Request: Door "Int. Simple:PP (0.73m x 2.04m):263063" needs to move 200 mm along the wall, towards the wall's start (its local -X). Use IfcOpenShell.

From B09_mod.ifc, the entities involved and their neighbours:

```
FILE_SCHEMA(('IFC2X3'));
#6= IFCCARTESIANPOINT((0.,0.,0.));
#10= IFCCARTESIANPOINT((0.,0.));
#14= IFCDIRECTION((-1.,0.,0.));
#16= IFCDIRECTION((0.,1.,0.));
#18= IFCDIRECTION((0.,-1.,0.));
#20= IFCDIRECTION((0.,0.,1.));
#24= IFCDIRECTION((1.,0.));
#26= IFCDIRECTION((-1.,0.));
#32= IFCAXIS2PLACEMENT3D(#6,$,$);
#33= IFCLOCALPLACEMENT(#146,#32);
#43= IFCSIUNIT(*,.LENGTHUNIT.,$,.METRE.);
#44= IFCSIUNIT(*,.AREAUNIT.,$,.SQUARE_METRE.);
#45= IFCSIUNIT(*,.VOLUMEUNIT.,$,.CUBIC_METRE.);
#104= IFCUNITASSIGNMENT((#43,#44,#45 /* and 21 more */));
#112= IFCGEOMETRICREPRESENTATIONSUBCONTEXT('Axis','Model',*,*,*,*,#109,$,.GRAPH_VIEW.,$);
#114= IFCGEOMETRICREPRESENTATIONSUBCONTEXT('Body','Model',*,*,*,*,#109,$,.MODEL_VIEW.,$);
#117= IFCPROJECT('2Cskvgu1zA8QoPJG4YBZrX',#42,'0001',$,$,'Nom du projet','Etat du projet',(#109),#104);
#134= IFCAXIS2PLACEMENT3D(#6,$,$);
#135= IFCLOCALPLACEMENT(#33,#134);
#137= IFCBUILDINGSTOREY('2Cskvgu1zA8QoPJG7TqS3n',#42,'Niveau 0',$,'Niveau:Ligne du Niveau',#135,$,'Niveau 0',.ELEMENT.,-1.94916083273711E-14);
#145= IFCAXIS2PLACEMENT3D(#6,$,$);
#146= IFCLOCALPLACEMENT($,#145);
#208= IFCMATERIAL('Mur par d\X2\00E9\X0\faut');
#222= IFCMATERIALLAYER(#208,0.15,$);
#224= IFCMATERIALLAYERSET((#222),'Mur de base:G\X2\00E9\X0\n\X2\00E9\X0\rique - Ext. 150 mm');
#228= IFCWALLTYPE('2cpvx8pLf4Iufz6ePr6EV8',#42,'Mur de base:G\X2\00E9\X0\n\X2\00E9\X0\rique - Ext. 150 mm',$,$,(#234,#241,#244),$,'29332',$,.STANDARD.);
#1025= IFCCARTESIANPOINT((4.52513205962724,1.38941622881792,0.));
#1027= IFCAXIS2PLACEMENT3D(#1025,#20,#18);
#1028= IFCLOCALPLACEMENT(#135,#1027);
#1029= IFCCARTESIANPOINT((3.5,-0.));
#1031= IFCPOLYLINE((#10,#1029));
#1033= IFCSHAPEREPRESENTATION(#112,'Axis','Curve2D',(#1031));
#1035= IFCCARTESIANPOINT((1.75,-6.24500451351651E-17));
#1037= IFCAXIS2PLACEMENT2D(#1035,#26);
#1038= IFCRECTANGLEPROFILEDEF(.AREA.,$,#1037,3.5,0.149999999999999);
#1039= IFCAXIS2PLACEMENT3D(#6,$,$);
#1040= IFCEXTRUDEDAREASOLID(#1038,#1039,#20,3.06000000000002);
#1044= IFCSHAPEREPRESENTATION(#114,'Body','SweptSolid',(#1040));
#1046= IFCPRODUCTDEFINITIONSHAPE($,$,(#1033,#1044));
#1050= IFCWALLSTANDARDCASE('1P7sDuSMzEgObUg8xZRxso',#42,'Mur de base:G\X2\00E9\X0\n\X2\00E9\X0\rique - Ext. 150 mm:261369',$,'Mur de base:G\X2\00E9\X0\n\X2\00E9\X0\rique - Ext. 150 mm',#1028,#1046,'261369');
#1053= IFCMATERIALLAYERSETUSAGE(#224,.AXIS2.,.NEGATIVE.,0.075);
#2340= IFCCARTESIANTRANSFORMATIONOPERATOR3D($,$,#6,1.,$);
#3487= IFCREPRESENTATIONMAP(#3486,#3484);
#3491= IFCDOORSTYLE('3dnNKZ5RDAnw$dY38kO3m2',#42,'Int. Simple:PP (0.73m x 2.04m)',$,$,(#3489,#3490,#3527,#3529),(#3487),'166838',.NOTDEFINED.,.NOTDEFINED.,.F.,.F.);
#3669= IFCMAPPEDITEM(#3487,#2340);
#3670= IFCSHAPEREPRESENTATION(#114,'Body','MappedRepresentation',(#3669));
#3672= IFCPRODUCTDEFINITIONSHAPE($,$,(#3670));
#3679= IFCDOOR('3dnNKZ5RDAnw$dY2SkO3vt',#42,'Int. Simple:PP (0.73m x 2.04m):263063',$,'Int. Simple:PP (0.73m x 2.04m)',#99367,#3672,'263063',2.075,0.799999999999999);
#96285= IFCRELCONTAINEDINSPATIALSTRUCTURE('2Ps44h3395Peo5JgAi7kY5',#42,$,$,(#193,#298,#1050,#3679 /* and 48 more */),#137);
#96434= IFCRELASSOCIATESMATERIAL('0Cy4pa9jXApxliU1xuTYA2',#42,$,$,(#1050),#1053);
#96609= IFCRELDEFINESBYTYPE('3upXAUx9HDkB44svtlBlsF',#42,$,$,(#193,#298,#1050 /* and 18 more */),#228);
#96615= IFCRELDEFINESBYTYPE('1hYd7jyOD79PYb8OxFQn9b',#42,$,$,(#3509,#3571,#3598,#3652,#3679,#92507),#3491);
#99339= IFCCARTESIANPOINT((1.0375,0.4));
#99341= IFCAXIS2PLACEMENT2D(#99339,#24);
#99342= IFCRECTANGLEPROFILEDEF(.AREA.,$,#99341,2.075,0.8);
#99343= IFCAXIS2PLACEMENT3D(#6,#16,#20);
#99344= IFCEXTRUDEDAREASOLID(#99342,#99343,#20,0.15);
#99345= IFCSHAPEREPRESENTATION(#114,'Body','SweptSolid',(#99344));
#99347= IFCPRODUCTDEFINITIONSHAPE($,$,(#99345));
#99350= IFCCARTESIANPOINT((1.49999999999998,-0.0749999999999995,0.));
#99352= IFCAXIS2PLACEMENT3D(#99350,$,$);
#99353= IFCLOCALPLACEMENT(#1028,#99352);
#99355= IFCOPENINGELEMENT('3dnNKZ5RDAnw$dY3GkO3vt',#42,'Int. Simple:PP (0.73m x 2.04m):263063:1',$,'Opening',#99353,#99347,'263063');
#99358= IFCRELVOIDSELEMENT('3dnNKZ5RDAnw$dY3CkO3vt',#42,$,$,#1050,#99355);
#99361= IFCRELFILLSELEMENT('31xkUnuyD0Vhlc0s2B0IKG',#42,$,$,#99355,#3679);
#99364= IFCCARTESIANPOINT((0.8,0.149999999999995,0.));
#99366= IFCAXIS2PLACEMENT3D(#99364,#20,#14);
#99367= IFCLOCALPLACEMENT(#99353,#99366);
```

```python
import ifcopenshell
import ifcopenshell.api.geometry
import ifcopenshell.util.placement

model = ifcopenshell.open("B09_mod.ifc")

door = model.by_guid("3dnNKZ5RDAnw$dY2SkO3vt")
opening = door.FillsVoids[0].RelatingOpeningElement
wall = opening.VoidsElements[0].RelatingBuildingElement

wall_matrix = ifcopenshell.util.placement.get_local_placement(wall.ObjectPlacement)
shift = wall_matrix[:3, 0] * -0.2
before = ifcopenshell.util.placement.get_local_placement(door.ObjectPlacement)[:3, 3].copy()

# The door is placed relative to its opening, so it follows when the opening moves.
matrix = ifcopenshell.util.placement.get_local_placement(opening.ObjectPlacement)
matrix[:3, 3] += shift
ifcopenshell.api.geometry.edit_object_placement(
    model, product=opening, matrix=matrix, is_si=False, should_transform_children=True
)

after = ifcopenshell.util.placement.get_local_placement(door.ObjectPlacement)[:3, 3]
print("door moved by", (after - before).round(3) + 0.0)

model.write("B09_mod_v2.ifc")
```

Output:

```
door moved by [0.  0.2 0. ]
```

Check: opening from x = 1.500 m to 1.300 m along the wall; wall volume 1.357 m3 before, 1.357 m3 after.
